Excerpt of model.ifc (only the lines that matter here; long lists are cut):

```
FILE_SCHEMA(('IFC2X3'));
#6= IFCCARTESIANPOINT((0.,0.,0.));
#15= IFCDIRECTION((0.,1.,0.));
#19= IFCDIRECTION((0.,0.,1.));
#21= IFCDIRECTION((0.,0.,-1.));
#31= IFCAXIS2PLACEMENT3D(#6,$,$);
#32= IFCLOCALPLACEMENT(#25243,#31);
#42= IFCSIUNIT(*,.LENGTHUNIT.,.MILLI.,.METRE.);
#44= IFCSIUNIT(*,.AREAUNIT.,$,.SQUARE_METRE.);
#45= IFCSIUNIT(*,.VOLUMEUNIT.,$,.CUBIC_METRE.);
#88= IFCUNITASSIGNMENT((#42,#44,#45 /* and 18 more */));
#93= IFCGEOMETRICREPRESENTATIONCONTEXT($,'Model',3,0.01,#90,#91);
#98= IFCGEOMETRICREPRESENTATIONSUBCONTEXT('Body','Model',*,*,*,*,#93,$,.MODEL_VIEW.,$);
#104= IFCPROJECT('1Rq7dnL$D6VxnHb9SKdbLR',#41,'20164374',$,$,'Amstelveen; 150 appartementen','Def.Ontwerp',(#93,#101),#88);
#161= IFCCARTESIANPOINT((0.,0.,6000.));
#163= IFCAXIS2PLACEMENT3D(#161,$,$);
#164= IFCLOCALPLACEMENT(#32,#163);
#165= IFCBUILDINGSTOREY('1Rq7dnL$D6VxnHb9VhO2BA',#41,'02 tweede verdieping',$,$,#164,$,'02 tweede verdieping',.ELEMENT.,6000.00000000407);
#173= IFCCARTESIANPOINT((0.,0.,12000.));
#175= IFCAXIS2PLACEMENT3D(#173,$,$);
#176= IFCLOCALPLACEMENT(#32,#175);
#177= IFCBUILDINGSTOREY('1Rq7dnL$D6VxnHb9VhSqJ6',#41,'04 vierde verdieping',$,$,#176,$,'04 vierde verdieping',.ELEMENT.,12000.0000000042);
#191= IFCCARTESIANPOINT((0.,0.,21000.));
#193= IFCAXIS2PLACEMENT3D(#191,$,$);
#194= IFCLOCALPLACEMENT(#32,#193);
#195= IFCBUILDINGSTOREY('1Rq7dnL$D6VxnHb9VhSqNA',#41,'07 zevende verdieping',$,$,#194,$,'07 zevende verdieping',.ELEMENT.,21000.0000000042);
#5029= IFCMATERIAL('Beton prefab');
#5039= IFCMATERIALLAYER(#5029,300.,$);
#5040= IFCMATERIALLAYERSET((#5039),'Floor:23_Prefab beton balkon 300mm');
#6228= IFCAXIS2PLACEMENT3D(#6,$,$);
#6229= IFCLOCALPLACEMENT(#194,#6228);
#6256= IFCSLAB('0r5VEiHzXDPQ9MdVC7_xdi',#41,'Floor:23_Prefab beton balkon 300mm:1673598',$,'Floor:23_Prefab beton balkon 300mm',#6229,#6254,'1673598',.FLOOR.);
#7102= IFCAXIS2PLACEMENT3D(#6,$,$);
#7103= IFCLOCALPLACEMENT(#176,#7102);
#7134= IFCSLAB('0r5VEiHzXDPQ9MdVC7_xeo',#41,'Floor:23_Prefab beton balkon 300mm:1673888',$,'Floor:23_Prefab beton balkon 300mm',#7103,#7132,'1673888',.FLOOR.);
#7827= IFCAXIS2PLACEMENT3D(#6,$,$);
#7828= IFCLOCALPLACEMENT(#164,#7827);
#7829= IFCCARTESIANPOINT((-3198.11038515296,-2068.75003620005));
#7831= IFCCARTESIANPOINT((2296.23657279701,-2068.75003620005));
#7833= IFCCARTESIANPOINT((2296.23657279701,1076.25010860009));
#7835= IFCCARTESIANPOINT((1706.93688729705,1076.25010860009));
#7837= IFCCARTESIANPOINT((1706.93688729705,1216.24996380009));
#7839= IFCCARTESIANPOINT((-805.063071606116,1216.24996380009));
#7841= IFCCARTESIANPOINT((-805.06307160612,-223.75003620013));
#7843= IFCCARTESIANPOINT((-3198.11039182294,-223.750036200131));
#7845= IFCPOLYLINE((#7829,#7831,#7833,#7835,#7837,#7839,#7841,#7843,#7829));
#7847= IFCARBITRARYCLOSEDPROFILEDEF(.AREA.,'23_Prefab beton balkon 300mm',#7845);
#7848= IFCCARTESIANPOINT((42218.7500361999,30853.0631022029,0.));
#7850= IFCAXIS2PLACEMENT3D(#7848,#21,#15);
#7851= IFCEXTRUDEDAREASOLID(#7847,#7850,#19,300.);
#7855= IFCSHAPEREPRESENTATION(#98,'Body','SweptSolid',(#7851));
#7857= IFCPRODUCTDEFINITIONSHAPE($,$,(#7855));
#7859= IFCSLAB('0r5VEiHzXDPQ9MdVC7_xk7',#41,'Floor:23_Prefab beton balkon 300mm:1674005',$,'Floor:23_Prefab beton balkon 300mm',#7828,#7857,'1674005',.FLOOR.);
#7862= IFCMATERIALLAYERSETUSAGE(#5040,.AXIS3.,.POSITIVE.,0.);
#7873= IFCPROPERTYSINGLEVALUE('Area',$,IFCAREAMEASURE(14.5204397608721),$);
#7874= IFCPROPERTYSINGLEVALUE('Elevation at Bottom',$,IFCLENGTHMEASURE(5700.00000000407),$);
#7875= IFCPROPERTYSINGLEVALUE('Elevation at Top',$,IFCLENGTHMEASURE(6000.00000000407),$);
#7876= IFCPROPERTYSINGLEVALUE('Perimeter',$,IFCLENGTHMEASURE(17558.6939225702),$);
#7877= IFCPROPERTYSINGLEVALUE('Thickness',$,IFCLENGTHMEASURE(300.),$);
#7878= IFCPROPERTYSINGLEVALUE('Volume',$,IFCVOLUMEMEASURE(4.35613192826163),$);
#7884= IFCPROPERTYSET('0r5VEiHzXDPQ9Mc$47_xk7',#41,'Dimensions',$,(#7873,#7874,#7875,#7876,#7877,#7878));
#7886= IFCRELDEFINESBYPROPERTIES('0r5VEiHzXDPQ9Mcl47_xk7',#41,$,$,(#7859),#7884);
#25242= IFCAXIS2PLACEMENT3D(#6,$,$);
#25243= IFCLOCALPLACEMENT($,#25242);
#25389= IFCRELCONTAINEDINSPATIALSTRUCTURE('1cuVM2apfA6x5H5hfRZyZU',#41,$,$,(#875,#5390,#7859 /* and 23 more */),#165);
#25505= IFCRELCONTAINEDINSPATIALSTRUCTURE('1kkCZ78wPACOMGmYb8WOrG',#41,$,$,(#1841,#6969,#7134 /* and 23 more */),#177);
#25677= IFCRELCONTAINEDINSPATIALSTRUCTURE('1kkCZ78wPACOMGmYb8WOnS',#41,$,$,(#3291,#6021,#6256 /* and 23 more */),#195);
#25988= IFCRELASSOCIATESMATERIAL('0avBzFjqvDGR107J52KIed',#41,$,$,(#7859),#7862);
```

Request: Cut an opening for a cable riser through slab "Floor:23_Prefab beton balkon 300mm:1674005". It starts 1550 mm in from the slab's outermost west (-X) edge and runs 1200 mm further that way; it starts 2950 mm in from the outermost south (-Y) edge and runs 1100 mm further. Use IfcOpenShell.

```python
import numpy as np
import ifcopenshell
import ifcopenshell.api.feature
import ifcopenshell.api.geometry
import ifcopenshell.api.pset
import ifcopenshell.api.root
import ifcopenshell.geom
import ifcopenshell.util.element
import ifcopenshell.util.placement
import ifcopenshell.util.representation
import ifcopenshell.util.shape
import ifcopenshell.util.unit

model = ifcopenshell.open("model.ifc")
unit_scale = ifcopenshell.util.unit.calculate_unit_scale(model)
area_scale = ifcopenshell.util.unit.calculate_unit_scale(model, "AREAUNIT")
volume_scale = ifcopenshell.util.unit.calculate_unit_scale(model, "VOLUMEUNIT")
settings = ifcopenshell.geom.settings()


def volume(element):
    """Net volume in cubic metres, openings subtracted."""
    shape = ifcopenshell.geom.create_shape(settings, element)
    return ifcopenshell.util.shape.get_volume(shape.geometry)


slab = model.by_id(7859)
before = volume(slab)

# Extent in the slab's own axes, in metres. The edges named are its -X and -Y sides.
slab_shape = ifcopenshell.geom.create_shape(settings, slab)
vertices = ifcopenshell.util.shape.get_vertices(slab_shape.geometry)
x_min, y_min, bottom = vertices.min(axis=0)
top = vertices[:, 2].max()

opening = ifcopenshell.api.root.create_entity(model, ifc_class="IfcOpeningElement", name="Cable riser opening")
context = ifcopenshell.util.representation.get_context(model, "Model", "Body", "MODEL_VIEW")
width, depth = 1.2, 1.1
outline = [(0.0, 0.0), (width, 0.0), (width, depth), (0.0, depth), (0.0, 0.0)]
# Overshoot both faces by 50 mm so the cut is clean.
shape = ifcopenshell.api.geometry.add_slab_representation(
    model, context=context, depth=top - bottom + 0.1, polyline=outline
)
ifcopenshell.api.geometry.assign_representation(model, product=opening, representation=shape)

matrix = ifcopenshell.util.placement.get_local_placement(slab.ObjectPlacement)
matrix[:, 3] = matrix @ np.append(np.array([x_min + 1.55, y_min + 2.95, bottom - 0.05]) / unit_scale, 1.0)
ifcopenshell.api.geometry.edit_object_placement(model, product=opening, matrix=matrix, is_si=False)
ifcopenshell.api.feature.add_feature(model, feature=opening, element=slab)

after = volume(slab)

# Update the slab's stored quantities.
pset = model.by_id(ifcopenshell.util.element.get_pset(slab, "Dimensions", should_inherit=False)["id"])
ifcopenshell.api.pset.edit_pset(model, pset=pset, properties={
    "Area": model.create_entity("IfcAreaMeasure", after / (top - bottom) / area_scale),
    "Volume": model.create_entity("IfcVolumeMeasure", after / volume_scale),
})

print(f"slab volume {before:.3f} -> {after:.3f} m3")

model.write("model_edited.ifc")
```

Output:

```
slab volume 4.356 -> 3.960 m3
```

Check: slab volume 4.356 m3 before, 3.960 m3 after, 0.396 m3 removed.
